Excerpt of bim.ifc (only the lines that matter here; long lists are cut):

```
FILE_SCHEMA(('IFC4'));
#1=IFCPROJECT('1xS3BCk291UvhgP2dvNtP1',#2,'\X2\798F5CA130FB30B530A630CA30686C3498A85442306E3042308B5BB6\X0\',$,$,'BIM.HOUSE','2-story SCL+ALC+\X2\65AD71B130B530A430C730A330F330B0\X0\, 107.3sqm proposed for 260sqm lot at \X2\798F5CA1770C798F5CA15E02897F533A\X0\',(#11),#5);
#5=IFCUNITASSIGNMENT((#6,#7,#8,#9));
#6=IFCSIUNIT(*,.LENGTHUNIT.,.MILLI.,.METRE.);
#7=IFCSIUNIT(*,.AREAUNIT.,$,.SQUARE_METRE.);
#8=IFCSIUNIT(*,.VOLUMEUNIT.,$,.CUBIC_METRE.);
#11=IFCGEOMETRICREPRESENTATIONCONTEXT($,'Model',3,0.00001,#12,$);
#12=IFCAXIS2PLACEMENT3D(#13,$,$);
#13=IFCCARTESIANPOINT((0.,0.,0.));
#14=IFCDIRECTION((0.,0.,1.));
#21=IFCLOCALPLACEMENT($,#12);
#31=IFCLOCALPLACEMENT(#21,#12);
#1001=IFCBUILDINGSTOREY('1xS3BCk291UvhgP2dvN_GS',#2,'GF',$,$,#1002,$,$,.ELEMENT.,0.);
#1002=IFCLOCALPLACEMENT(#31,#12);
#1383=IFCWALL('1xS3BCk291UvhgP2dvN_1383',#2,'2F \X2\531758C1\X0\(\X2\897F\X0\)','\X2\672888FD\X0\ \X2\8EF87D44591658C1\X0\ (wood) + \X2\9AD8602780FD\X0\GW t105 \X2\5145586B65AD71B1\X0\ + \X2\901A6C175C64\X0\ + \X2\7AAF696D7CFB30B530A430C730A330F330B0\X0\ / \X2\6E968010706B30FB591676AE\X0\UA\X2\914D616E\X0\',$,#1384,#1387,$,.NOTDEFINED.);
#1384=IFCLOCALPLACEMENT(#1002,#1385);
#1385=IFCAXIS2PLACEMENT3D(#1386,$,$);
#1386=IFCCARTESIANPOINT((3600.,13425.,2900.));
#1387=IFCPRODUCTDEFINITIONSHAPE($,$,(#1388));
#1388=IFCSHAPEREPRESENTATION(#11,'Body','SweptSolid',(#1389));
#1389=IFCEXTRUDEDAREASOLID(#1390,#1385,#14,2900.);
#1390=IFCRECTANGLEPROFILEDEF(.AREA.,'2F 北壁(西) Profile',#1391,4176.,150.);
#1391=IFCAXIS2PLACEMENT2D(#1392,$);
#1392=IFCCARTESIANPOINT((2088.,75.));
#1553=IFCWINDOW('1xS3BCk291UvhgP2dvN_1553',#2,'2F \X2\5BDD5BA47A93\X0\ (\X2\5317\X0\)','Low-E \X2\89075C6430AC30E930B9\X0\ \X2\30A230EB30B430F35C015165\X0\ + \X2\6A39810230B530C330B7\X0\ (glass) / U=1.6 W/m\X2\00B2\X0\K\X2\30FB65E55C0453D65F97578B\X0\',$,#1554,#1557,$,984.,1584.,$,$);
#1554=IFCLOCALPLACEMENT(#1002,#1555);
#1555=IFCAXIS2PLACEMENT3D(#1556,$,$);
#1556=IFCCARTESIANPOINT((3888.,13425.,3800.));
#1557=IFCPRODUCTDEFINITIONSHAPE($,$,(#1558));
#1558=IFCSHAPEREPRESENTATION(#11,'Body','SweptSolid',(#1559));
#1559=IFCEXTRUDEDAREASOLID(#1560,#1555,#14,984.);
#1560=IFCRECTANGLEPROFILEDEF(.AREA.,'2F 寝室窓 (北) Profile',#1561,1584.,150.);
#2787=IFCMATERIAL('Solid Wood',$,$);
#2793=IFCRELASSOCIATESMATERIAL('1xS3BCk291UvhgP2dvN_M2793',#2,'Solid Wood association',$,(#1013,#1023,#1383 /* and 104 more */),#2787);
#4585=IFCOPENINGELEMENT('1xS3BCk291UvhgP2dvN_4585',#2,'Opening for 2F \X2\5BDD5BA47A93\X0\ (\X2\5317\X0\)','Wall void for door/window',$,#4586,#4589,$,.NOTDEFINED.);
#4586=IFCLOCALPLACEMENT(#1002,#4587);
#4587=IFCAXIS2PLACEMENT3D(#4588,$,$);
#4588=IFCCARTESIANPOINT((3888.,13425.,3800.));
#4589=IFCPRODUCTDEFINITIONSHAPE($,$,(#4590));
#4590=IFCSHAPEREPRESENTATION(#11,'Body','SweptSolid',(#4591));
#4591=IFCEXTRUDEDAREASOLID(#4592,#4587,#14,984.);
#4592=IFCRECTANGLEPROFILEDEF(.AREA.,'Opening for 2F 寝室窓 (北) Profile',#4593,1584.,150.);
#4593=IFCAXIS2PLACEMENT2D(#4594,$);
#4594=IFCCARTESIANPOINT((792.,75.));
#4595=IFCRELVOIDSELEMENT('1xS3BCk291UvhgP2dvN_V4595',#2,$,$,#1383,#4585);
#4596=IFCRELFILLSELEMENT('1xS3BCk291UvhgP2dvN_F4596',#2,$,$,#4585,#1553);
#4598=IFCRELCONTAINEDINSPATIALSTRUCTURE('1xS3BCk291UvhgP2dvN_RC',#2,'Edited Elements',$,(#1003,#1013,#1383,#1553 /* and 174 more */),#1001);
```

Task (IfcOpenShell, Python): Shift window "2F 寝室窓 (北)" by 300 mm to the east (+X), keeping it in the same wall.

```python
import ifcopenshell
import ifcopenshell.api.geometry
import ifcopenshell.util.placement
import ifcopenshell.util.unit

model = ifcopenshell.open("bim.ifc")
unit_scale = ifcopenshell.util.unit.calculate_unit_scale(model)

window = model.by_guid("1xS3BCk291UvhgP2dvN_1553")
opening = window.FillsVoids[0].RelatingOpeningElement
wall = opening.VoidsElements[0].RelatingBuildingElement

wall_matrix = ifcopenshell.util.placement.get_local_placement(wall.ObjectPlacement)
shift = wall_matrix[:3, 0] * 0.3 / unit_scale
before = ifcopenshell.util.placement.get_local_placement(window.ObjectPlacement)[:3, 3].copy()

# The window is not placed relative to its opening, so move both.
for product in (opening, window):
    matrix = ifcopenshell.util.placement.get_local_placement(product.ObjectPlacement)
    matrix[:3, 3] += shift
    ifcopenshell.api.geometry.edit_object_placement(model, product=product, matrix=matrix, is_si=False)

after = ifcopenshell.util.placement.get_local_placement(window.ObjectPlacement)[:3, 3]
print("window moved by", (after - before).round(3) + 0.0)

model.write("bim-out.ifc")
```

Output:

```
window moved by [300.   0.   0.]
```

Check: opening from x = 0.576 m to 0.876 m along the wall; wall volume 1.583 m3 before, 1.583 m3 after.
